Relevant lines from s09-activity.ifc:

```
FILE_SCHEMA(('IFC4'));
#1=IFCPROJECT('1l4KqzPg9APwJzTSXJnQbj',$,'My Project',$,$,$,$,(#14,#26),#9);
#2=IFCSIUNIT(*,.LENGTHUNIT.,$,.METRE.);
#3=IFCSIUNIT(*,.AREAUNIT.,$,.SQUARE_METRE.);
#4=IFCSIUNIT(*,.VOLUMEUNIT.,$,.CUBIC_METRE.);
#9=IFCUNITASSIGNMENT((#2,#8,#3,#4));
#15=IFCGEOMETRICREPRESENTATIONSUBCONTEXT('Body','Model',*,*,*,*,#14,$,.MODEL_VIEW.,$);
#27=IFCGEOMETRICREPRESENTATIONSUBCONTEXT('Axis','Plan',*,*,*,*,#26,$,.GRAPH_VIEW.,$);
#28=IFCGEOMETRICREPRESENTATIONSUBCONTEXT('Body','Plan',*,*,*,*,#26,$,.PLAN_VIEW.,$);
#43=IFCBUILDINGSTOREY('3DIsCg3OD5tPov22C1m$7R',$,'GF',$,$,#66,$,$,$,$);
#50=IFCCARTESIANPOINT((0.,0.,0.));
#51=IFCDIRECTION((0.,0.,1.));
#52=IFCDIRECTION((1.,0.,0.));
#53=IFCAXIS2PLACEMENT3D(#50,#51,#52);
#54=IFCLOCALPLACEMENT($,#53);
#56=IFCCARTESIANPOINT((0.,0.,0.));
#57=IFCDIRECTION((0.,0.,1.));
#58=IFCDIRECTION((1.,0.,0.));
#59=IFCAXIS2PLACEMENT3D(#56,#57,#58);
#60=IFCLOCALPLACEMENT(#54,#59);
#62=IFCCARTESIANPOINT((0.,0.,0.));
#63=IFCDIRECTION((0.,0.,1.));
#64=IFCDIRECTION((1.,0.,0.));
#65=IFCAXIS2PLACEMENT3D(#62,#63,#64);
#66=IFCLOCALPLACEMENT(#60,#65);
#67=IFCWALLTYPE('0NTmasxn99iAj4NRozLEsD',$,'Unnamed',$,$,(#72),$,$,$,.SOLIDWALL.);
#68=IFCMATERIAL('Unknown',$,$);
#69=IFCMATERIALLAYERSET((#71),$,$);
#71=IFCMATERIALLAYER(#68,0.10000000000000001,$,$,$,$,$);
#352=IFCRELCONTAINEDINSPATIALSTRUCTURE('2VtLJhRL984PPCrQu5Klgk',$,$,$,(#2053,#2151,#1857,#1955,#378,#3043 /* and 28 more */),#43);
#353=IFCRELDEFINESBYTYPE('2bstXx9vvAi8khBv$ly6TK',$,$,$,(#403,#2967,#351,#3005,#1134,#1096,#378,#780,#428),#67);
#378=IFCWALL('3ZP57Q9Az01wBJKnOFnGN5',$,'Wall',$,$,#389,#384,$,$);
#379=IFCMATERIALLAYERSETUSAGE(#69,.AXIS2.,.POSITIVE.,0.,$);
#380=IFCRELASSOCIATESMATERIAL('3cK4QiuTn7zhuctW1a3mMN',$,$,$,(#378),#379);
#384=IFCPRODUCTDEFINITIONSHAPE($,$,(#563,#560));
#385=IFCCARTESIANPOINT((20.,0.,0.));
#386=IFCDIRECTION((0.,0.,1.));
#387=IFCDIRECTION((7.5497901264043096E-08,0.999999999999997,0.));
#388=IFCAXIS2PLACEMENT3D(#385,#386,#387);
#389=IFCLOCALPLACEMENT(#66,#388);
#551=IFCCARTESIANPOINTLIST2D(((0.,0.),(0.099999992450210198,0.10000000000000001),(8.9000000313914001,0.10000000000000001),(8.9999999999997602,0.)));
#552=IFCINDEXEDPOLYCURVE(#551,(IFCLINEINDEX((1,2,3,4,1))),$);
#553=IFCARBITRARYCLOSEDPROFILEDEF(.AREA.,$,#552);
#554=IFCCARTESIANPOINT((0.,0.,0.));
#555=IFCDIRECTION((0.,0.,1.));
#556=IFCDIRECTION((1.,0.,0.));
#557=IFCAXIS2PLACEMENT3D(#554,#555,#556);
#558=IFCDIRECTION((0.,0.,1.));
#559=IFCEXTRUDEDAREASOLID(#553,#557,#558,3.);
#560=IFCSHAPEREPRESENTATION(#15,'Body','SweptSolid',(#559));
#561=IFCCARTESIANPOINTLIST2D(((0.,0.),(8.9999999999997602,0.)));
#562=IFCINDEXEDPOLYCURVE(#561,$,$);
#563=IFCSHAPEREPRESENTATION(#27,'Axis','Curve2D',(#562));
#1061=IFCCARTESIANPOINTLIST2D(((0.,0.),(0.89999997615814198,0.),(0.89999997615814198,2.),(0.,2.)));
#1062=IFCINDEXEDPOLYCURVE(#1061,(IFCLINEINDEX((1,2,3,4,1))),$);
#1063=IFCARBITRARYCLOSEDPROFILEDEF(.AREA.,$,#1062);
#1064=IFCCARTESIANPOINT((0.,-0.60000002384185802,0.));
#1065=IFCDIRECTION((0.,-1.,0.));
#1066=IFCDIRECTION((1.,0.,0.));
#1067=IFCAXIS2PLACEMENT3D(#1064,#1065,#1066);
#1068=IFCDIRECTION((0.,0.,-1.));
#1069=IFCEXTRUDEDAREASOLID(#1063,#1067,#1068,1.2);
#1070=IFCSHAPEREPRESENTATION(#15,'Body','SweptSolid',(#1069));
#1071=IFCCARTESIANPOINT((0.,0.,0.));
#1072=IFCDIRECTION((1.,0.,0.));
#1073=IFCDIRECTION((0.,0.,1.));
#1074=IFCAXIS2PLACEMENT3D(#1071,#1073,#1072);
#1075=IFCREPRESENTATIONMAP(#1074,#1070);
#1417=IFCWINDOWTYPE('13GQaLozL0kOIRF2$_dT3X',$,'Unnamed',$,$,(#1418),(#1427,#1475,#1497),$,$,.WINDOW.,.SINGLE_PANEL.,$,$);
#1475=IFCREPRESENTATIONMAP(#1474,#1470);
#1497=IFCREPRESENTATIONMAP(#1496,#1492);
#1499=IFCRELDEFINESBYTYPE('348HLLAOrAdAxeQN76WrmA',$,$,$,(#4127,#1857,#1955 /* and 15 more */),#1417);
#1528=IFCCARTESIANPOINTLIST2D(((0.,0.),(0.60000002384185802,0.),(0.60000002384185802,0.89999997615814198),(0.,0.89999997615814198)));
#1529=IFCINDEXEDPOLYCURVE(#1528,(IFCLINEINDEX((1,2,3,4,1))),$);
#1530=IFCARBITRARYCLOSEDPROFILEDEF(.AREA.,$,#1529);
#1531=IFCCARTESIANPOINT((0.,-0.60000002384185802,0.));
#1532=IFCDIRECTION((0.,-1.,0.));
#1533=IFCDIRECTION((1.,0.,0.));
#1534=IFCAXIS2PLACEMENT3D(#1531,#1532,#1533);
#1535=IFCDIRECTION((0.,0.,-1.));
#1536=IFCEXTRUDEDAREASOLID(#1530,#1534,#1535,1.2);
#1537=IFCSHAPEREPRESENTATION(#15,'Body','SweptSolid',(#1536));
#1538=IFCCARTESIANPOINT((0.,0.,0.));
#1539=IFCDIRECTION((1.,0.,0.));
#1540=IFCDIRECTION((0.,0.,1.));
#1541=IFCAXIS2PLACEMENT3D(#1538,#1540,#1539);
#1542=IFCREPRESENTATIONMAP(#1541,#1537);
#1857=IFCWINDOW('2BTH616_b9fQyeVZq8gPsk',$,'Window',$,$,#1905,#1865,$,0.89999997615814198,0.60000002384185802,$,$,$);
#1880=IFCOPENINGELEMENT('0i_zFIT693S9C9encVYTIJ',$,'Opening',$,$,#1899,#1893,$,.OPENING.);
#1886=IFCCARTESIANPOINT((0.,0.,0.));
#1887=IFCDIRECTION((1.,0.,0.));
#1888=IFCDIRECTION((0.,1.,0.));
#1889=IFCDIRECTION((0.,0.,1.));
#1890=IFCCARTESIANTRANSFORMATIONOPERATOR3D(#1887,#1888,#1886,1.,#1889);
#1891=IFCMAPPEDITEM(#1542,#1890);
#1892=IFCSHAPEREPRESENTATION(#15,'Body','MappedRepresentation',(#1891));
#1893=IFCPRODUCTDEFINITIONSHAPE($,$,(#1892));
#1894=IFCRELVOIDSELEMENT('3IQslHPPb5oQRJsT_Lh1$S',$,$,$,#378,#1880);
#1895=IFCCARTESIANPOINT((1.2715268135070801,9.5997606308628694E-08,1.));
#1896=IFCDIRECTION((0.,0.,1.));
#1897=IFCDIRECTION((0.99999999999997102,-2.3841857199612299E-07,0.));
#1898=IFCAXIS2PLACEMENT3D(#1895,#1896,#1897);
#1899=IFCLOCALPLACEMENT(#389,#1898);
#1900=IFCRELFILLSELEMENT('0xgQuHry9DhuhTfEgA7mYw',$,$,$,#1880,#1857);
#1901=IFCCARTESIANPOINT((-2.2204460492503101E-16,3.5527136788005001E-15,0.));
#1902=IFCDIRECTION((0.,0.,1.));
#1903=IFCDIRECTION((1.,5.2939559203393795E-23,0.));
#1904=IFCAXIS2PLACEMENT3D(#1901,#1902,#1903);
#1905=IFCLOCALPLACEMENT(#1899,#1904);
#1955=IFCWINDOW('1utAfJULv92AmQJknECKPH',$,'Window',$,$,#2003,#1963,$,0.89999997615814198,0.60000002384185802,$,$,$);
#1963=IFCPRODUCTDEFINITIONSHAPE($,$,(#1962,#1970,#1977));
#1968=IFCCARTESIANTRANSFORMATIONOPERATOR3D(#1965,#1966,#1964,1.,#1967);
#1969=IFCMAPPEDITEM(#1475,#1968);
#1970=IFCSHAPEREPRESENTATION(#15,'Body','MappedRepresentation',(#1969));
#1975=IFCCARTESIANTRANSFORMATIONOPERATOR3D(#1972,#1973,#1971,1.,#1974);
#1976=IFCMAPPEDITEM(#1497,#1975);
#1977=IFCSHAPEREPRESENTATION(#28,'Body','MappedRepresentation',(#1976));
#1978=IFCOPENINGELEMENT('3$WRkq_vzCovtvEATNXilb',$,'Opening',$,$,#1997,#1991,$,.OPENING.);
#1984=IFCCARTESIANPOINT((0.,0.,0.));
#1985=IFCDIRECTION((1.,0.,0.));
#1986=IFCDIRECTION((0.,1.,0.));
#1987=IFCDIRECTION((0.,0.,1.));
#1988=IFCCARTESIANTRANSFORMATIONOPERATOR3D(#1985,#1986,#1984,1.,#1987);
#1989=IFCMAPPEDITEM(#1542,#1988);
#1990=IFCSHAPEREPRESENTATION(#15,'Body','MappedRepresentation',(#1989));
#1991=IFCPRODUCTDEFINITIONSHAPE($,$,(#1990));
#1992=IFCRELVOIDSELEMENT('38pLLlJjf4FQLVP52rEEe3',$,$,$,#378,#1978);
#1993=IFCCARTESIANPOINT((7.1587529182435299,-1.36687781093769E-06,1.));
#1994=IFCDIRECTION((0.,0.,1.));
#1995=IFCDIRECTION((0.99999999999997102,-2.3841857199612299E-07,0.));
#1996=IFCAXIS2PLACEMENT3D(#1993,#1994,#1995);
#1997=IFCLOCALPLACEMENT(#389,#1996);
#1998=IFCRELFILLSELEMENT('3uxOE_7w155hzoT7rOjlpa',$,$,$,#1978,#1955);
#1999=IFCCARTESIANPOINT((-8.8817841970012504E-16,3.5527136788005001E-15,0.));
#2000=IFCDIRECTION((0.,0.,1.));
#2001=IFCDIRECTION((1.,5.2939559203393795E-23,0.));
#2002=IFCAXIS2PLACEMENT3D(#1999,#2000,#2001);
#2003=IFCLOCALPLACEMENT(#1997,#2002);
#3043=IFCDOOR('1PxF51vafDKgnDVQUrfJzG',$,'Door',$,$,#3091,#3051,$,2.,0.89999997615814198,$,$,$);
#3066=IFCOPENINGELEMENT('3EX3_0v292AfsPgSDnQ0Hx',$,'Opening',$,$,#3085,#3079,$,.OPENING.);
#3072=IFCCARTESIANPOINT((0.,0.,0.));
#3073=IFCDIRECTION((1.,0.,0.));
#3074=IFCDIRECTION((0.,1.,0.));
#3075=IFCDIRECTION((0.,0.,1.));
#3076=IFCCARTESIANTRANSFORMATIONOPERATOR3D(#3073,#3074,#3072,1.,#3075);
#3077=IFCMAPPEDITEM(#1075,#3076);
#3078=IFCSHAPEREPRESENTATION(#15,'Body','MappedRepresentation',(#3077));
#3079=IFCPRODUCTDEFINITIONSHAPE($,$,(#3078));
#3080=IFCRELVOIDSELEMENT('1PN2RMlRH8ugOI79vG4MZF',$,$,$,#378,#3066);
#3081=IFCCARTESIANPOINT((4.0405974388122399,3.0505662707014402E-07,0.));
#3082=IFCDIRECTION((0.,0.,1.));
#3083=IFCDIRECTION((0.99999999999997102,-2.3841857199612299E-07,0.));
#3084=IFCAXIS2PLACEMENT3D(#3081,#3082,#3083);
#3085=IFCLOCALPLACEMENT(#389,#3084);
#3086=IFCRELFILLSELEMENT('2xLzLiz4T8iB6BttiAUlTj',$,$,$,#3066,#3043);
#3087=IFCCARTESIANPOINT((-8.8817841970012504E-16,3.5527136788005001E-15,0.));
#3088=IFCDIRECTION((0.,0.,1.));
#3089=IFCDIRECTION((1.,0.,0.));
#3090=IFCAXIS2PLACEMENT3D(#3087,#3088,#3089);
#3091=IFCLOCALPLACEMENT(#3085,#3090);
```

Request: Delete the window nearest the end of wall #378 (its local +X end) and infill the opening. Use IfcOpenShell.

```python
import ifcopenshell
import ifcopenshell.api.feature
import ifcopenshell.api.root
import ifcopenshell.geom
import ifcopenshell.util.shape

model = ifcopenshell.open("s09-activity.ifc")
settings = ifcopenshell.geom.settings()


def volume(element):
    """Net volume in cubic metres, openings subtracted."""
    shape = ifcopenshell.geom.create_shape(settings, element)
    return ifcopenshell.util.shape.get_volume(shape.geometry)


window = model.by_guid("1utAfJULv92AmQJknECKPH")
opening = window.FillsVoids[0].RelatingOpeningElement
wall = opening.VoidsElements[0].RelatingBuildingElement
before = volume(wall)

ifcopenshell.api.root.remove_product(model, product=window)
ifcopenshell.api.feature.remove_feature(model, feature=opening)

after = volume(wall)

print(f"wall volume {before:.3f} -> {after:.3f} m3")

model.write("s09-activity-out.ifc")
```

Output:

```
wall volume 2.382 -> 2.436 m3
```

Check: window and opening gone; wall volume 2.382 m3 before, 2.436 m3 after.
